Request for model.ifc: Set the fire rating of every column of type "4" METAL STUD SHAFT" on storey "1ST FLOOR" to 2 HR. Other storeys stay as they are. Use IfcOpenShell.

First a look at what the model holds.

```python
import ifcopenshell
import ifcopenshell.util.element

model = ifcopenshell.open("model.ifc")
print(model.schema)
storey = next(s for s in model.by_type("IfcBuildingStorey") if s.Name == "1ST FLOOR")
columns = [e for e in ifcopenshell.util.element.get_decomposition(storey) if e.is_a("IfcColumn")]
seen = {}
for e in columns:
    element_type = ifcopenshell.util.element.get_type(e)
    key = (element_type.Name if element_type != e and element_type else None, ifcopenshell.util.element.get_pset(e, "Pset_ColumnCommon", "FireRating"))
    seen[key] = seen.get(key, 0) + 1
for (name, value), count in sorted(seen.items(), key=str):
    print(count, "x", name, "|", value)
```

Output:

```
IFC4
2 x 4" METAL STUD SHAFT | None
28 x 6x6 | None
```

```python
import ifcopenshell
import ifcopenshell.api.pset
import ifcopenshell.util.element

model = ifcopenshell.open("model.ifc")

storey = next(s for s in model.by_type("IfcBuildingStorey") if s.Name == "1ST FLOOR")
columns = [e for e in ifcopenshell.util.element.get_decomposition(storey) if e.is_a("IfcColumn")]

count = 0
for e in columns:
    element_type = ifcopenshell.util.element.get_type(e)
    if element_type in (None, e) or element_type.Name != '4" METAL STUD SHAFT':
        continue
    # add_pset returns the element's existing set when there is one.
    pset = ifcopenshell.api.pset.add_pset(model, product=e, name="Pset_ColumnCommon")
    ifcopenshell.api.pset.edit_pset(model, pset=pset, properties={"FireRating": "2 HR"})
    count += 1

print(count, "columns updated")

model.write("model_rev.ifc")
```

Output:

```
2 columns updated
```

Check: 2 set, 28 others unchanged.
